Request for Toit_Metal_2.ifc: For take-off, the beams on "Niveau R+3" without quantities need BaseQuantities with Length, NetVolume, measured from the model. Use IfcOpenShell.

First a look at what the model holds.

```python
import ifcopenshell
import ifcopenshell.util.element
import ifcopenshell.util.unit

model = ifcopenshell.open("Toit_Metal_2.ifc")
print(model.schema)
for unit_type in ("LENGTHUNIT", "AREAUNIT", "VOLUMEUNIT"):
    print(unit_type, ifcopenshell.util.unit.calculate_unit_scale(model, unit_type))
storey = next(s for s in model.by_type("IfcBuildingStorey") if s.Name == "Niveau R+3")
beams = [e for e in ifcopenshell.util.element.get_decomposition(storey) if e.is_a("IfcBeam")]
for e in sorted(beams, key=lambda e: e.id()):
    print(e.id(), e.is_a(), e.Name, list(ifcopenshell.util.element.get_psets(e, qtos_only=True)), sep=" | ")
```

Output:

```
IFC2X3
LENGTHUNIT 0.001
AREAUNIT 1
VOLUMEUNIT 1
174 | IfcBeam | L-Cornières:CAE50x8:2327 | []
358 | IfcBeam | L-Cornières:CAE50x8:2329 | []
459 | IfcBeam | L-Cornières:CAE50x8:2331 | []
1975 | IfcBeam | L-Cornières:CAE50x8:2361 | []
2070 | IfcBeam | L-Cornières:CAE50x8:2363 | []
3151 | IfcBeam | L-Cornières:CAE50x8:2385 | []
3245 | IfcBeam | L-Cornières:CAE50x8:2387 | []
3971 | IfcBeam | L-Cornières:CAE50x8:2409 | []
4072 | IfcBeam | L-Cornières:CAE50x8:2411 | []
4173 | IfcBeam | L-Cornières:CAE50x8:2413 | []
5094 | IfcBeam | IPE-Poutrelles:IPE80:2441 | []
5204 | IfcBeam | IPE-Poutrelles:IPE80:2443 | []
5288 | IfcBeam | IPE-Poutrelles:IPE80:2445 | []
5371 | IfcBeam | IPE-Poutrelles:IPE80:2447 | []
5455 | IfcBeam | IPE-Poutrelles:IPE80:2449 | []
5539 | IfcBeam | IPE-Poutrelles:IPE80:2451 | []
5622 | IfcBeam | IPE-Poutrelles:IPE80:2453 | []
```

```python
import ifcopenshell
import ifcopenshell.api.pset
import ifcopenshell.geom
import ifcopenshell.util.element
import ifcopenshell.util.shape
import ifcopenshell.util.unit

model = ifcopenshell.open("Toit_Metal_2.ifc")
unit_scale = ifcopenshell.util.unit.calculate_unit_scale(model)
volume_scale = ifcopenshell.util.unit.calculate_unit_scale(model, "VOLUMEUNIT")
settings = ifcopenshell.geom.settings()

storey = next(s for s in model.by_type("IfcBuildingStorey") if s.Name == "Niveau R+3")
beams = [e for e in ifcopenshell.util.element.get_decomposition(storey) if e.is_a("IfcBeam")]

for e in sorted(beams, key=lambda e: e.id()):
    if ifcopenshell.util.element.get_psets(e, qtos_only=True, should_inherit=False):
        continue
    # Geometry comes back in metres, in the element's own axes.
    shape = ifcopenshell.geom.create_shape(settings, e)
    values = {
        "Length": ifcopenshell.util.shape.get_max_xyz(shape.geometry) / unit_scale,
        "NetVolume": ifcopenshell.util.shape.get_volume(shape.geometry) / volume_scale,
    }
    qto = ifcopenshell.api.pset.add_qto(model, product=e, name="BaseQuantities")
    ifcopenshell.api.pset.edit_qto(model, qto=qto, properties=values)
    print(e.id(), {k: round(v, 3) for k, v in values.items()})

model.write("Toit_Metal_2_edited.ifc")
```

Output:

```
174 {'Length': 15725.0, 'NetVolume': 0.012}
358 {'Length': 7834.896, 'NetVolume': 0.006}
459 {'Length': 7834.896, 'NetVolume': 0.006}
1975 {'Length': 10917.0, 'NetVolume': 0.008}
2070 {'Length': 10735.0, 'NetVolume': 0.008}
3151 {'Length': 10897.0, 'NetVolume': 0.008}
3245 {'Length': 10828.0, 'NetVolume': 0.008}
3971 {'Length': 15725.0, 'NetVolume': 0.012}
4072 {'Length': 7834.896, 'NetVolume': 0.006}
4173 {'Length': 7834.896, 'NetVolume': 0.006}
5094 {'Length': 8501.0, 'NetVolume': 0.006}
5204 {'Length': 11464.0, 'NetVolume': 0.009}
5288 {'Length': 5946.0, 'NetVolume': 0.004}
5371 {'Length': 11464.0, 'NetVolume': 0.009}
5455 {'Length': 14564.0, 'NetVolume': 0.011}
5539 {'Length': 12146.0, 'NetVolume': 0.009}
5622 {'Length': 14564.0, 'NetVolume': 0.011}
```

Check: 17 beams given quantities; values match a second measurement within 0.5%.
